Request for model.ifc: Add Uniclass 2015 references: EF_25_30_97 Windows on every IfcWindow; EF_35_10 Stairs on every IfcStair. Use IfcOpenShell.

First a look at what the model holds.

```python
import ifcopenshell

model = ifcopenshell.open("model.ifc")
print(model.schema)
print("classifications:", [c.Name for c in model.by_type("IfcClassification")])
for ifc_class in ("IfcDoor", "IfcRoof", "IfcStair", "IfcWall", "IfcWindow"):
    print(ifc_class, len(model.by_type(ifc_class)))
```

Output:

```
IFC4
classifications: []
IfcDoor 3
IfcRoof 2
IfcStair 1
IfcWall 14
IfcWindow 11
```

```python
import ifcopenshell
import ifcopenshell.api.classification

model = ifcopenshell.open("model.ifc")

system = ifcopenshell.api.classification.add_classification(model, classification="Uniclass 2015")

codes = {
    "IfcWindow": ("EF_25_30_97", "Windows"),
    "IfcStair": ("EF_35_10", "Stairs"),
}
for ifc_class, (code, name) in codes.items():
    products = model.by_type(ifc_class)
    ifcopenshell.api.classification.add_reference(
        model, products=products, classification=system, identification=code, name=name
    )
    print(code, len(products))

model.write("model-out.ifc")
```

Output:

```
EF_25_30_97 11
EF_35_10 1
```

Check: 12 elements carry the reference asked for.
